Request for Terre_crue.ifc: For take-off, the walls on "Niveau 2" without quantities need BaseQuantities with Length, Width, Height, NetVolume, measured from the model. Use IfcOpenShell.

First a look at what the model holds.

```python
import ifcopenshell
import ifcopenshell.util.element
import ifcopenshell.util.unit

model = ifcopenshell.open("Terre_crue.ifc")
print(model.schema)
for unit_type in ("LENGTHUNIT", "AREAUNIT", "VOLUMEUNIT"):
    print(unit_type, ifcopenshell.util.unit.calculate_unit_scale(model, unit_type))
storey = next(s for s in model.by_type("IfcBuildingStorey") if s.Name == "Niveau 2")
walls = [e for e in ifcopenshell.util.element.get_decomposition(storey) if e.is_a("IfcWall")]
for e in sorted(walls, key=lambda e: e.id()):
    print(e.id(), e.is_a(), e.Name, list(ifcopenshell.util.element.get_psets(e, qtos_only=True)), sep=" | ")
```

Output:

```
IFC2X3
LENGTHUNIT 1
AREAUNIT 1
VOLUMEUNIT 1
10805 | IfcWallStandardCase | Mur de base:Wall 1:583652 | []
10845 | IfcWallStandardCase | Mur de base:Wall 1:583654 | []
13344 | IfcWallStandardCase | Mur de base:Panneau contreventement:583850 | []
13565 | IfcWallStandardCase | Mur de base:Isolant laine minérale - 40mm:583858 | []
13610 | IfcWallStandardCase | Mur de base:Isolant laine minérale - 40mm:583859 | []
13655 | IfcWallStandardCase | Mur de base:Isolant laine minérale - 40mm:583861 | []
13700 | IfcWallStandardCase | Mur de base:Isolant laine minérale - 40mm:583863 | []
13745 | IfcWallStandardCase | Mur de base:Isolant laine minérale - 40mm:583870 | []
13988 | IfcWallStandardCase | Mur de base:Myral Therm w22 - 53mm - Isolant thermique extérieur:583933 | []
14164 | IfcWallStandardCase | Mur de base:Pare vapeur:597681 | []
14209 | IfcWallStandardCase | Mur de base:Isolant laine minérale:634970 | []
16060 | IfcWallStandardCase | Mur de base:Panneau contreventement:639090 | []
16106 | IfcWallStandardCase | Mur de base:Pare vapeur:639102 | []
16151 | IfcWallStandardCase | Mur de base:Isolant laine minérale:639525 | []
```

```python
import ifcopenshell
import ifcopenshell.api.pset
import ifcopenshell.geom
import ifcopenshell.util.element
import ifcopenshell.util.shape
import ifcopenshell.util.unit

model = ifcopenshell.open("Terre_crue.ifc")
unit_scale = ifcopenshell.util.unit.calculate_unit_scale(model)
volume_scale = ifcopenshell.util.unit.calculate_unit_scale(model, "VOLUMEUNIT")
settings = ifcopenshell.geom.settings()

storey = next(s for s in model.by_type("IfcBuildingStorey") if s.Name == "Niveau 2")
walls = [e for e in ifcopenshell.util.element.get_decomposition(storey) if e.is_a("IfcWall")]

for e in sorted(walls, key=lambda e: e.id()):
    if ifcopenshell.util.element.get_psets(e, qtos_only=True, should_inherit=False):
        continue
    # Geometry comes back in metres, in the element's own axes.
    shape = ifcopenshell.geom.create_shape(settings, e)
    values = {
        "Length": ifcopenshell.util.shape.get_x(shape.geometry) / unit_scale,
        "Width": ifcopenshell.util.shape.get_y(shape.geometry) / unit_scale,
        "Height": ifcopenshell.util.shape.get_z(shape.geometry) / unit_scale,
        "NetVolume": ifcopenshell.util.shape.get_volume(shape.geometry) / volume_scale,
    }
    qto = ifcopenshell.api.pset.add_qto(model, product=e, name="BaseQuantities")
    ifcopenshell.api.pset.edit_qto(model, qto=qto, properties=values)
    print(e.id(), {k: round(v, 3) for k, v in values.items()})

model.write("Terre_crue_v2.ifc")
```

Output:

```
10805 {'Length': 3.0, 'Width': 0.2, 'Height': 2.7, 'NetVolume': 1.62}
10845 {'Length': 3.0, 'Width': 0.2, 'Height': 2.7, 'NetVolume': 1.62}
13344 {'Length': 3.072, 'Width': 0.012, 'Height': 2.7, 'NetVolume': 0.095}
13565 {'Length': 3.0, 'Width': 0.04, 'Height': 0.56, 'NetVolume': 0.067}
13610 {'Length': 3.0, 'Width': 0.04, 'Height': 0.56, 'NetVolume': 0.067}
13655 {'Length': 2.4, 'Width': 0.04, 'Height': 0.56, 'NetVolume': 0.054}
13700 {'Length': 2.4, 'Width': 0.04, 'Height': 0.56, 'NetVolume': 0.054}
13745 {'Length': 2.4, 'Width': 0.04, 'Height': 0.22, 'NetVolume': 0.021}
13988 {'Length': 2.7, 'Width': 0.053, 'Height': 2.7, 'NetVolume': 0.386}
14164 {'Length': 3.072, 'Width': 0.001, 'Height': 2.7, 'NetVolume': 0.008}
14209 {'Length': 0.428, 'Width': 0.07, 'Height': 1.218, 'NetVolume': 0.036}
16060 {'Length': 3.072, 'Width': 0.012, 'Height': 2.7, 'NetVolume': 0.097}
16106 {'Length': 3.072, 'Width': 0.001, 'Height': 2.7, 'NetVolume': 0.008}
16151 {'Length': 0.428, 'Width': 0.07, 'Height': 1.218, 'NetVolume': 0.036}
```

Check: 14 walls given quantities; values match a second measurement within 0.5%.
